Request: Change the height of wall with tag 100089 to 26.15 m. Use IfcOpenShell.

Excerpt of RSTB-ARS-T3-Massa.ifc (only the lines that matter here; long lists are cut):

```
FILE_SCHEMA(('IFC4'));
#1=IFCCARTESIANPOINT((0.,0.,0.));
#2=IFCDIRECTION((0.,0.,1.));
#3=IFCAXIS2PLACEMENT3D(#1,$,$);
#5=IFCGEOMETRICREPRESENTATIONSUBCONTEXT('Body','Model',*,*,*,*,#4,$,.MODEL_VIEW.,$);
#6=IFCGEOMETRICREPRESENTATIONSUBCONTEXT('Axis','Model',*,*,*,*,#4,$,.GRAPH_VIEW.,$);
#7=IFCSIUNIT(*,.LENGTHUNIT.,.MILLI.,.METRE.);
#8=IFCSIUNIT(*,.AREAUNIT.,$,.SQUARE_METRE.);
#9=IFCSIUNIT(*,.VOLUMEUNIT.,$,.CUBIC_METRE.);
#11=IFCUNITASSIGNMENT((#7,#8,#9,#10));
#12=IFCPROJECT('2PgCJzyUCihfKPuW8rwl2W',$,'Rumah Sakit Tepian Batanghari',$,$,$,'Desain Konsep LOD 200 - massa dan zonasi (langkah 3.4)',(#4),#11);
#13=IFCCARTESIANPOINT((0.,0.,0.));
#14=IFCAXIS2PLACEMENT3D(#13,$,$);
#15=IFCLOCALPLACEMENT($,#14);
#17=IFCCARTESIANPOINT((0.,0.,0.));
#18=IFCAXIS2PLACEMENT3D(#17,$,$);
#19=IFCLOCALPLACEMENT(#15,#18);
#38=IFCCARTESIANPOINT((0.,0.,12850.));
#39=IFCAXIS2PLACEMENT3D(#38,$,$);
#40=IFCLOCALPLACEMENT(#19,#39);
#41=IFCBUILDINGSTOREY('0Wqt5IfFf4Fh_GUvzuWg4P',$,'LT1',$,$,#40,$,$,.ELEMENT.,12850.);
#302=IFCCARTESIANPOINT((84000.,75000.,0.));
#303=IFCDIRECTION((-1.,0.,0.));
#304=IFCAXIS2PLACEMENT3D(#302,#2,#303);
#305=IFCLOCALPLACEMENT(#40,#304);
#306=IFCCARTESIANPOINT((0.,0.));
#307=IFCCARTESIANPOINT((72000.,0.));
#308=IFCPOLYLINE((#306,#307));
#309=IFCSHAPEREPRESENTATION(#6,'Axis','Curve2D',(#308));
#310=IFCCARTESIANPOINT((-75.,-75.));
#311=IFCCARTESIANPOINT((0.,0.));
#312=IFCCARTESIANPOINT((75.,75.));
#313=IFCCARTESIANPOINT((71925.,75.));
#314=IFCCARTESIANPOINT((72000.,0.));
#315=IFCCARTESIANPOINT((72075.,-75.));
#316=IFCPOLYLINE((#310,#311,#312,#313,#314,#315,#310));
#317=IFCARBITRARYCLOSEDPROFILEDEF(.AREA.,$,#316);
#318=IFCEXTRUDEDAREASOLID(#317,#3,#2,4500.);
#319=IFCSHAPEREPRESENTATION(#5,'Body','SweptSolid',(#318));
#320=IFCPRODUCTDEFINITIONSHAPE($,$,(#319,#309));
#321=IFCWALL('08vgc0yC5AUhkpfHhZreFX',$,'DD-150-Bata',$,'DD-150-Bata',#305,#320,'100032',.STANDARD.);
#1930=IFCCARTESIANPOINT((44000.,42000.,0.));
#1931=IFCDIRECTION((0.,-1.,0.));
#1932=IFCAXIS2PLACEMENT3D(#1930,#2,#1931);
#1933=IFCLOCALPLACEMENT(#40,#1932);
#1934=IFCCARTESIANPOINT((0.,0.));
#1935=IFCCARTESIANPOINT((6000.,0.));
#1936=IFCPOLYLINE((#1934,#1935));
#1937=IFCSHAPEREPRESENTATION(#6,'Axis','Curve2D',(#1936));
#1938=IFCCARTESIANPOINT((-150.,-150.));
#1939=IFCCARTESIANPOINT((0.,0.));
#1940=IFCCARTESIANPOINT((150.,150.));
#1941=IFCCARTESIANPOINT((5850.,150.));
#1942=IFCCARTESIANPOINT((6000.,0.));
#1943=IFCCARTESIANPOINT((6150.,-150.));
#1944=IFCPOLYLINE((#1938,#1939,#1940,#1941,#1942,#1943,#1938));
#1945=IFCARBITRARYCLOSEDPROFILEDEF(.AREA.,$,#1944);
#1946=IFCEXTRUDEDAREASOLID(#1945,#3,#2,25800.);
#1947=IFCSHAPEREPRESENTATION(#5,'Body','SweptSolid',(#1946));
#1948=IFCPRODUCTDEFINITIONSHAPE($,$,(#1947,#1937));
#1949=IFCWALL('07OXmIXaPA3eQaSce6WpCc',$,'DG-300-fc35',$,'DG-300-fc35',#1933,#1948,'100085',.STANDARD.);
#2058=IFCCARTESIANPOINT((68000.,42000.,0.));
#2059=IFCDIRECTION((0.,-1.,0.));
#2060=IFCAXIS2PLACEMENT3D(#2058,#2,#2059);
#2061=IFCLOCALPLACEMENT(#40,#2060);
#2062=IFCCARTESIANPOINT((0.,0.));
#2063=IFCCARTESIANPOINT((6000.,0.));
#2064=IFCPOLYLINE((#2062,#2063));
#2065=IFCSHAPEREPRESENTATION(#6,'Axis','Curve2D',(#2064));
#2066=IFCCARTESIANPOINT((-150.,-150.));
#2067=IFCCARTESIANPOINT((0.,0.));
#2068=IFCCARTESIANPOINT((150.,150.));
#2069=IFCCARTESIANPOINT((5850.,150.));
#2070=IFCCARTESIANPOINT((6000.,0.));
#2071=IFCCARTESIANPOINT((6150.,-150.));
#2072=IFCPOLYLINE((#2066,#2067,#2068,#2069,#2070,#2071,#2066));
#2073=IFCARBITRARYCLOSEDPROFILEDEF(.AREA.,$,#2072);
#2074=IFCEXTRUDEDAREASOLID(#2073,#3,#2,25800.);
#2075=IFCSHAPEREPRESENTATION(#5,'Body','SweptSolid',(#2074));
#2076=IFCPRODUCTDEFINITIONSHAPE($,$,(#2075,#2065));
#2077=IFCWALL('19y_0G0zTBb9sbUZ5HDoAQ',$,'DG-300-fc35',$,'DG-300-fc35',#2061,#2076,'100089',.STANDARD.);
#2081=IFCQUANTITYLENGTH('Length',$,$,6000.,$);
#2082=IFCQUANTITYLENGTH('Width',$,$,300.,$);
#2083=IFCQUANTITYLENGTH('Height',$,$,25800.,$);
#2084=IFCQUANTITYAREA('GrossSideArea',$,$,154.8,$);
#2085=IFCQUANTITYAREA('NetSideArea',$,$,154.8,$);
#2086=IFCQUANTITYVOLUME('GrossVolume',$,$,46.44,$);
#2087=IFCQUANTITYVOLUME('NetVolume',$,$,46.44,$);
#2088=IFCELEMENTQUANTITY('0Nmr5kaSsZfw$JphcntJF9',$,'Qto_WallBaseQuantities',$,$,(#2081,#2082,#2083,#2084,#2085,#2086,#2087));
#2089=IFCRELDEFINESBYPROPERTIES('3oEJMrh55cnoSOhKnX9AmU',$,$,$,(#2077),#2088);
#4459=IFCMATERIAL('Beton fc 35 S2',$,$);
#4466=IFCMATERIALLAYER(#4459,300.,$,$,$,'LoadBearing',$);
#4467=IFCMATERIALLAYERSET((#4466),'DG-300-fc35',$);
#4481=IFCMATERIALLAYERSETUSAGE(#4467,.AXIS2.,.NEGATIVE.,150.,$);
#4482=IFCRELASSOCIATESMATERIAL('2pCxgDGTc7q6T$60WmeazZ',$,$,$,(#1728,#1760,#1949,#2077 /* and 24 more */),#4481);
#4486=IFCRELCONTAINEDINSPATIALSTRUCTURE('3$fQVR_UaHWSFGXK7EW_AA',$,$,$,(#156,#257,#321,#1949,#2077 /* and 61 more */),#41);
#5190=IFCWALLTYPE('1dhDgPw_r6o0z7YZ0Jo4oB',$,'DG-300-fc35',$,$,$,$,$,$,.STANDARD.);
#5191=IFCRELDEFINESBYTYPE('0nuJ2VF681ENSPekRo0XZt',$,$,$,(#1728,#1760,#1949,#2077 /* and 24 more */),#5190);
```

```python
import ifcopenshell
import ifcopenshell.api.pset
import ifcopenshell.geom
import ifcopenshell.util.element
import ifcopenshell.util.representation
import ifcopenshell.util.shape
import ifcopenshell.util.unit

model = ifcopenshell.open("RSTB-ARS-T3-Massa.ifc")
unit_scale = ifcopenshell.util.unit.calculate_unit_scale(model)
area_scale = ifcopenshell.util.unit.calculate_unit_scale(model, "AREAUNIT")
volume_scale = ifcopenshell.util.unit.calculate_unit_scale(model, "VOLUMEUNIT")
settings = ifcopenshell.geom.settings()


def volume(element):
    """Net volume in cubic metres, openings subtracted."""
    shape = ifcopenshell.geom.create_shape(settings, element)
    return ifcopenshell.util.shape.get_volume(shape.geometry)


wall = model.by_guid("19y_0G0zTBb9sbUZ5HDoAQ")
before = volume(wall)

body = ifcopenshell.util.representation.get_representation(wall, "Model", "Body")
solid = body.Items[0]
old_height = solid.Depth
solid.Depth = 26.15 / unit_scale
after = volume(wall)
thickness = 0.3  # wall thickness in metres

# Update the stored height, areas and volumes.
qto = model.by_id(ifcopenshell.util.element.get_pset(wall, "Qto_WallBaseQuantities", should_inherit=False)["id"])
ifcopenshell.api.pset.edit_qto(model, qto=qto, properties={
    "Height": solid.Depth,
    "GrossSideArea": ifcopenshell.util.element.get_pset(wall, "Qto_WallBaseQuantities", "GrossSideArea") * solid.Depth / old_height,
    "NetSideArea": after / thickness / area_scale,
    "GrossVolume": ifcopenshell.util.element.get_pset(wall, "Qto_WallBaseQuantities", "GrossVolume") * solid.Depth / old_height,
    "NetVolume": after / volume_scale,
})

print(f"height {old_height:g} -> {solid.Depth:g}, volume {before:.3f} -> {after:.3f} m3")

model.write("RSTB-ARS-T3-Massa_edited.ifc")
```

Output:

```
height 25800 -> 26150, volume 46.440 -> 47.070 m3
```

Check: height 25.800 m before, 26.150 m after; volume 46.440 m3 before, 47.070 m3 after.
